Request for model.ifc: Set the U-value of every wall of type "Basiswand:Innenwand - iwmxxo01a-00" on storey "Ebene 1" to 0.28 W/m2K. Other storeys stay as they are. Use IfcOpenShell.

First a look at what the model holds.

```python
import ifcopenshell
import ifcopenshell.util.element

model = ifcopenshell.open("model.ifc")
print(model.schema)
storey = next(s for s in model.by_type("IfcBuildingStorey") if s.Name == "Ebene 1")
walls = [e for e in ifcopenshell.util.element.get_decomposition(storey) if e.is_a("IfcWall")]
seen = {}
for e in walls:
    element_type = ifcopenshell.util.element.get_type(e)
    key = (element_type.Name if element_type != e and element_type else None, ifcopenshell.util.element.get_pset(e, "Pset_WallCommon", "ThermalTransmittance"))
    seen[key] = seen.get(key, 0) + 1
for (name, value), count in sorted(seen.items(), key=str):
    print(count, "x", name, "|", value)
```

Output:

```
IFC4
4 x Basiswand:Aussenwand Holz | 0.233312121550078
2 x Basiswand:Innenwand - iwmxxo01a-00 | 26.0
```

```python
import ifcopenshell
import ifcopenshell.api.pset
import ifcopenshell.util.element

model = ifcopenshell.open("model.ifc")

storey = next(s for s in model.by_type("IfcBuildingStorey") if s.Name == "Ebene 1")
walls = [e for e in ifcopenshell.util.element.get_decomposition(storey) if e.is_a("IfcWall")]

count = 0
for e in walls:
    element_type = ifcopenshell.util.element.get_type(e)
    if element_type in (None, e) or element_type.Name != "Basiswand:Innenwand - iwmxxo01a-00":
        continue
    # add_pset returns the element's existing set when there is one.
    pset = ifcopenshell.api.pset.add_pset(model, product=e, name="Pset_WallCommon")
    ifcopenshell.api.pset.edit_pset(model, pset=pset, properties={"ThermalTransmittance": 0.28})
    count += 1

print(count, "walls updated")

model.write("model_edited.ifc")
```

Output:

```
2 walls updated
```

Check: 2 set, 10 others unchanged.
